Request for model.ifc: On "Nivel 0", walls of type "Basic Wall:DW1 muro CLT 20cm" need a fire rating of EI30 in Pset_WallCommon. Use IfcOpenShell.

First a look at what the model holds.

```python
import ifcopenshell
import ifcopenshell.util.element

model = ifcopenshell.open("model.ifc")
print(model.schema)
storey = next(s for s in model.by_type("IfcBuildingStorey") if s.Name == "Nivel 0")
walls = [e for e in ifcopenshell.util.element.get_decomposition(storey) if e.is_a("IfcWall")]
seen = {}
for e in walls:
    element_type = ifcopenshell.util.element.get_type(e)
    key = (element_type.Name if element_type != e and element_type else None, ifcopenshell.util.element.get_pset(e, "Pset_WallCommon", "FireRating"))
    seen[key] = seen.get(key, 0) + 1
for (name, value), count in sorted(seen.items(), key=str):
    print(count, "x", name, "|", value)
```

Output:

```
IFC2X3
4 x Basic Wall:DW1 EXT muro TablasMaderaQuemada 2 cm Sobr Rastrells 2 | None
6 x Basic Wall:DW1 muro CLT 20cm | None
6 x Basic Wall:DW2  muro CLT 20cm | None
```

```python
import ifcopenshell
import ifcopenshell.api.pset
import ifcopenshell.util.element

model = ifcopenshell.open("model.ifc")

storey = next(s for s in model.by_type("IfcBuildingStorey") if s.Name == "Nivel 0")
walls = [e for e in ifcopenshell.util.element.get_decomposition(storey) if e.is_a("IfcWall")]

count = 0
for e in walls:
    element_type = ifcopenshell.util.element.get_type(e)
    if element_type in (None, e) or element_type.Name != "Basic Wall:DW1 muro CLT 20cm":
        continue
    # add_pset returns the element's existing set when there is one.
    pset = ifcopenshell.api.pset.add_pset(model, product=e, name="Pset_WallCommon")
    ifcopenshell.api.pset.edit_pset(model, pset=pset, properties={"FireRating": "EI30"})
    count += 1

print(count, "walls updated")

model.write("model_rev.ifc")
```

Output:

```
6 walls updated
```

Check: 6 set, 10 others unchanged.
